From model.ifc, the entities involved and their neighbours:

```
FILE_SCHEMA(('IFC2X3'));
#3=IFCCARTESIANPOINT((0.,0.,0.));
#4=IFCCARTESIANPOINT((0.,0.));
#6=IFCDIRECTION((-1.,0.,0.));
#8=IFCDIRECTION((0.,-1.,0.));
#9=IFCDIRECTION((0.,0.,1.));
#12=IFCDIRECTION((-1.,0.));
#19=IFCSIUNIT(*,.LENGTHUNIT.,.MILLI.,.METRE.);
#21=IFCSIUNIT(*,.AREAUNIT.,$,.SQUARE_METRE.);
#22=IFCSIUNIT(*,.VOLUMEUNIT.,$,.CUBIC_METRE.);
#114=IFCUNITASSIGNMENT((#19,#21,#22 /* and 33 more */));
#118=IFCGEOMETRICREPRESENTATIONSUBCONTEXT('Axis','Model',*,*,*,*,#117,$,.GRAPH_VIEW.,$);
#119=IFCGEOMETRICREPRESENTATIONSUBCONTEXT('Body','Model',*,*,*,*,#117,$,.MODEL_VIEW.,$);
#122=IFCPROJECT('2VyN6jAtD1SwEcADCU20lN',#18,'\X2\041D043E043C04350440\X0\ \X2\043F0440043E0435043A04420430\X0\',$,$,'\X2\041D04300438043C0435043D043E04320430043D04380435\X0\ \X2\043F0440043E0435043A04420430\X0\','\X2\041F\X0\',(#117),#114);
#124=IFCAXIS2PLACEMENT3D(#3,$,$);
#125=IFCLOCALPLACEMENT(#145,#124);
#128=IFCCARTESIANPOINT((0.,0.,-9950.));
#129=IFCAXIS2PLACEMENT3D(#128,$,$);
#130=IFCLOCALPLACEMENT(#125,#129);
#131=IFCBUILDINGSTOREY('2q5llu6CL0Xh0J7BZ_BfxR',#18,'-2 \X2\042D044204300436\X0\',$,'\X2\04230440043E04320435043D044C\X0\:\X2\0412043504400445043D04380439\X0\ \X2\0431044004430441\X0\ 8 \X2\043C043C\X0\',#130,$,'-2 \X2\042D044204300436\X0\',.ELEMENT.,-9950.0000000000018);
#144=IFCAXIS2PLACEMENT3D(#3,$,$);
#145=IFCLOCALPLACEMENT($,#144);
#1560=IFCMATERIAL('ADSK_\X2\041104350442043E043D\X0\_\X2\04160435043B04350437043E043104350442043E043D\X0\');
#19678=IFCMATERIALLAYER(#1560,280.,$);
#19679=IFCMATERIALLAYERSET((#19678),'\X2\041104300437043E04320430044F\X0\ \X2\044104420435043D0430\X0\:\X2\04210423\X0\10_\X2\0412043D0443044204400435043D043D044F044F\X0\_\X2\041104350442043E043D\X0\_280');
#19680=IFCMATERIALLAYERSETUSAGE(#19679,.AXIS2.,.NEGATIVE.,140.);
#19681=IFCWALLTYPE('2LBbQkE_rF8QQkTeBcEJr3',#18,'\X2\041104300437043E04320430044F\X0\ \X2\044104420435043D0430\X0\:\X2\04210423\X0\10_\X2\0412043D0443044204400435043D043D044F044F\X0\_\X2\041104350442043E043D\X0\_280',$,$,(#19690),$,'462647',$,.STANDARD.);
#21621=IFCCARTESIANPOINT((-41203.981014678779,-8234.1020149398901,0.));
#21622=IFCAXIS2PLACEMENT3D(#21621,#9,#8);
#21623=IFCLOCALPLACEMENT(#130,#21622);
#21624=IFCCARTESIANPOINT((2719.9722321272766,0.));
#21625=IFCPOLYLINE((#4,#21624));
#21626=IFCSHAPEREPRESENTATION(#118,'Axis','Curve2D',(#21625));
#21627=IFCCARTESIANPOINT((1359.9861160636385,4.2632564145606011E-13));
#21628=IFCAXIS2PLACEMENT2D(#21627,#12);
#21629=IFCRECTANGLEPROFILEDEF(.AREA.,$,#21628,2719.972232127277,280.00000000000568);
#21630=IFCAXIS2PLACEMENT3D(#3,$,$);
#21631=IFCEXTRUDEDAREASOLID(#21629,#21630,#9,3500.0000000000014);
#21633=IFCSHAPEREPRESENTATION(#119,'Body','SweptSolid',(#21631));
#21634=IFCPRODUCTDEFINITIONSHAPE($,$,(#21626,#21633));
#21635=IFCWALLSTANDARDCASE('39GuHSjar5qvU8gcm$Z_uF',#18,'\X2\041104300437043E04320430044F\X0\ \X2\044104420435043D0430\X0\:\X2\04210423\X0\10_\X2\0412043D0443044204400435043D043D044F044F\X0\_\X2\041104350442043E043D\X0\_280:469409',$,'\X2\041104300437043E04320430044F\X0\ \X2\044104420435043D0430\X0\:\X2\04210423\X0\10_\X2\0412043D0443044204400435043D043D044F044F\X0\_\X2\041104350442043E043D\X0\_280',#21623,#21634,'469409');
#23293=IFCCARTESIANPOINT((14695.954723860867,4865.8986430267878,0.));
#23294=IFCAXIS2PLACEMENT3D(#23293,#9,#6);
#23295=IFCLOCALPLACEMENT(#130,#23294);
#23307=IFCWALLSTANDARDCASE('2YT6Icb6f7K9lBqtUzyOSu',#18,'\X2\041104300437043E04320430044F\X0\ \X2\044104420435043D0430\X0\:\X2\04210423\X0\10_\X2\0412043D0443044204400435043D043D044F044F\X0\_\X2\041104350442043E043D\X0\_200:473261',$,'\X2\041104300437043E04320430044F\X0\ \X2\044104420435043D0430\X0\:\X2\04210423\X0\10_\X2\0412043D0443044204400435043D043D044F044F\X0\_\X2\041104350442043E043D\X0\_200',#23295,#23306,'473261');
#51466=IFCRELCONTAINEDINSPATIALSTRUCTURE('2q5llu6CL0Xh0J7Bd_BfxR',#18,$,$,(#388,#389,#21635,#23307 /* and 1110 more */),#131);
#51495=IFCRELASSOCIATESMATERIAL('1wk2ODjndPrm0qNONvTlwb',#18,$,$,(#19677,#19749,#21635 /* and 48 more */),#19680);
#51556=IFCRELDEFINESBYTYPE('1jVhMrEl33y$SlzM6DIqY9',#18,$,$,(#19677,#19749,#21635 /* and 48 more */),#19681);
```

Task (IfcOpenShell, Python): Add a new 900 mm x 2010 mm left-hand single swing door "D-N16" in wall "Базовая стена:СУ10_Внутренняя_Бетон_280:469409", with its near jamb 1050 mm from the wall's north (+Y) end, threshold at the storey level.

```python
import numpy as np
import ifcopenshell
import ifcopenshell.api.feature
import ifcopenshell.api.geometry
import ifcopenshell.api.root
import ifcopenshell.api.spatial
import ifcopenshell.api.type
import ifcopenshell.geom
import ifcopenshell.util.element
import ifcopenshell.util.placement
import ifcopenshell.util.representation
import ifcopenshell.util.shape
import ifcopenshell.util.unit

model = ifcopenshell.open("model.ifc")
unit_scale = ifcopenshell.util.unit.calculate_unit_scale(model)
settings = ifcopenshell.geom.settings()


def volume(element):
    """Net volume in cubic metres, openings subtracted."""
    shape = ifcopenshell.geom.create_shape(settings, element)
    return ifcopenshell.util.shape.get_volume(shape.geometry)


wall = model.by_guid("39GuHSjar5qvU8gcm$Z_uF")
storey = ifcopenshell.util.element.get_container(wall, ifc_class="IfcBuildingStorey")
context = ifcopenshell.util.representation.get_context(model, "Model", "Body", "MODEL_VIEW")
before = volume(wall)

width, height, from_end, sill = 0.9, 2.01, 1.05, 0.0  # metres

# The wall runs along its own X axis, and the end named is its -X end.
wall_shape = ifcopenshell.geom.create_shape(settings, wall)
x, y, z = ifcopenshell.util.shape.get_vertices(wall_shape.geometry).T
start = x.min() + from_end
face, thickness = float(y.min()), float(y.max() - y.min())
wall_matrix = ifcopenshell.util.placement.get_local_placement(wall.ObjectPlacement)
level = ifcopenshell.util.placement.get_local_placement(storey.ObjectPlacement)[2, 3]


def in_wall(x, y):
    """Placement at x, y metres in the wall's axes, at sill height."""
    matrix = wall_matrix.copy()
    matrix[:, 3] = wall_matrix @ np.array([x / unit_scale, y / unit_scale, 0.0, 1.0])
    matrix[2, 3] = level + sill / unit_scale
    return matrix


# Opening: a box that overshoots both wall faces by 50 mm.
opening = ifcopenshell.api.root.create_entity(model, ifc_class="IfcOpeningElement")
box = ifcopenshell.api.geometry.add_wall_representation(
    model, context=context, length=width, height=height, thickness=thickness + 0.1
)
ifcopenshell.api.geometry.assign_representation(model, product=opening, representation=box)
ifcopenshell.api.geometry.edit_object_placement(model, product=opening, matrix=in_wall(start, face - 0.05), is_si=False)
ifcopenshell.api.feature.add_feature(model, feature=opening, element=wall)

door = ifcopenshell.api.root.create_entity(model, ifc_class="IfcDoor", name="D-N16")
door.OverallWidth, door.OverallHeight = width / unit_scale, height / unit_scale
body = ifcopenshell.api.geometry.add_door_representation(
    model,
    context=context,
    overall_width=door.OverallWidth,
    overall_height=door.OverallHeight,
    operation_type="SINGLE_SWING_LEFT",
    lining_properties={"LiningDepth": thickness / unit_scale, "ThresholdDepth": thickness / unit_scale},
)
ifcopenshell.api.geometry.assign_representation(model, product=door, representation=body)
ifcopenshell.api.spatial.assign_container(model, products=[door], relating_structure=storey)
fills = ifcopenshell.api.feature.add_filling(model, opening=opening, element=door)
fills.OwnerHistory = door.OwnerHistory  # required in IFC2X3

# IFC2X3 keeps the operation on the door style.
style = ifcopenshell.api.root.create_entity(model, ifc_class="IfcDoorStyle", name="D-N16")
style.OperationType, style.ConstructionType = "SINGLE_SWING_LEFT", "NOTDEFINED"
style.ParameterTakesPrecedence = style.Sizeable = False
ifcopenshell.api.type.assign_type(model, related_objects=[door], relating_type=style)

# The lining spans the wall, so the door starts at the wall face.
ifcopenshell.api.geometry.edit_object_placement(model, product=door, matrix=in_wall(start, face), is_si=False)

after = volume(wall)

print(f"wall volume {before:.3f} -> {after:.3f} m3")

model.write("model_rev.ifc")
```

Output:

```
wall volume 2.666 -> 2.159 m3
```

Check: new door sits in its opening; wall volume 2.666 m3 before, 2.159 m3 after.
